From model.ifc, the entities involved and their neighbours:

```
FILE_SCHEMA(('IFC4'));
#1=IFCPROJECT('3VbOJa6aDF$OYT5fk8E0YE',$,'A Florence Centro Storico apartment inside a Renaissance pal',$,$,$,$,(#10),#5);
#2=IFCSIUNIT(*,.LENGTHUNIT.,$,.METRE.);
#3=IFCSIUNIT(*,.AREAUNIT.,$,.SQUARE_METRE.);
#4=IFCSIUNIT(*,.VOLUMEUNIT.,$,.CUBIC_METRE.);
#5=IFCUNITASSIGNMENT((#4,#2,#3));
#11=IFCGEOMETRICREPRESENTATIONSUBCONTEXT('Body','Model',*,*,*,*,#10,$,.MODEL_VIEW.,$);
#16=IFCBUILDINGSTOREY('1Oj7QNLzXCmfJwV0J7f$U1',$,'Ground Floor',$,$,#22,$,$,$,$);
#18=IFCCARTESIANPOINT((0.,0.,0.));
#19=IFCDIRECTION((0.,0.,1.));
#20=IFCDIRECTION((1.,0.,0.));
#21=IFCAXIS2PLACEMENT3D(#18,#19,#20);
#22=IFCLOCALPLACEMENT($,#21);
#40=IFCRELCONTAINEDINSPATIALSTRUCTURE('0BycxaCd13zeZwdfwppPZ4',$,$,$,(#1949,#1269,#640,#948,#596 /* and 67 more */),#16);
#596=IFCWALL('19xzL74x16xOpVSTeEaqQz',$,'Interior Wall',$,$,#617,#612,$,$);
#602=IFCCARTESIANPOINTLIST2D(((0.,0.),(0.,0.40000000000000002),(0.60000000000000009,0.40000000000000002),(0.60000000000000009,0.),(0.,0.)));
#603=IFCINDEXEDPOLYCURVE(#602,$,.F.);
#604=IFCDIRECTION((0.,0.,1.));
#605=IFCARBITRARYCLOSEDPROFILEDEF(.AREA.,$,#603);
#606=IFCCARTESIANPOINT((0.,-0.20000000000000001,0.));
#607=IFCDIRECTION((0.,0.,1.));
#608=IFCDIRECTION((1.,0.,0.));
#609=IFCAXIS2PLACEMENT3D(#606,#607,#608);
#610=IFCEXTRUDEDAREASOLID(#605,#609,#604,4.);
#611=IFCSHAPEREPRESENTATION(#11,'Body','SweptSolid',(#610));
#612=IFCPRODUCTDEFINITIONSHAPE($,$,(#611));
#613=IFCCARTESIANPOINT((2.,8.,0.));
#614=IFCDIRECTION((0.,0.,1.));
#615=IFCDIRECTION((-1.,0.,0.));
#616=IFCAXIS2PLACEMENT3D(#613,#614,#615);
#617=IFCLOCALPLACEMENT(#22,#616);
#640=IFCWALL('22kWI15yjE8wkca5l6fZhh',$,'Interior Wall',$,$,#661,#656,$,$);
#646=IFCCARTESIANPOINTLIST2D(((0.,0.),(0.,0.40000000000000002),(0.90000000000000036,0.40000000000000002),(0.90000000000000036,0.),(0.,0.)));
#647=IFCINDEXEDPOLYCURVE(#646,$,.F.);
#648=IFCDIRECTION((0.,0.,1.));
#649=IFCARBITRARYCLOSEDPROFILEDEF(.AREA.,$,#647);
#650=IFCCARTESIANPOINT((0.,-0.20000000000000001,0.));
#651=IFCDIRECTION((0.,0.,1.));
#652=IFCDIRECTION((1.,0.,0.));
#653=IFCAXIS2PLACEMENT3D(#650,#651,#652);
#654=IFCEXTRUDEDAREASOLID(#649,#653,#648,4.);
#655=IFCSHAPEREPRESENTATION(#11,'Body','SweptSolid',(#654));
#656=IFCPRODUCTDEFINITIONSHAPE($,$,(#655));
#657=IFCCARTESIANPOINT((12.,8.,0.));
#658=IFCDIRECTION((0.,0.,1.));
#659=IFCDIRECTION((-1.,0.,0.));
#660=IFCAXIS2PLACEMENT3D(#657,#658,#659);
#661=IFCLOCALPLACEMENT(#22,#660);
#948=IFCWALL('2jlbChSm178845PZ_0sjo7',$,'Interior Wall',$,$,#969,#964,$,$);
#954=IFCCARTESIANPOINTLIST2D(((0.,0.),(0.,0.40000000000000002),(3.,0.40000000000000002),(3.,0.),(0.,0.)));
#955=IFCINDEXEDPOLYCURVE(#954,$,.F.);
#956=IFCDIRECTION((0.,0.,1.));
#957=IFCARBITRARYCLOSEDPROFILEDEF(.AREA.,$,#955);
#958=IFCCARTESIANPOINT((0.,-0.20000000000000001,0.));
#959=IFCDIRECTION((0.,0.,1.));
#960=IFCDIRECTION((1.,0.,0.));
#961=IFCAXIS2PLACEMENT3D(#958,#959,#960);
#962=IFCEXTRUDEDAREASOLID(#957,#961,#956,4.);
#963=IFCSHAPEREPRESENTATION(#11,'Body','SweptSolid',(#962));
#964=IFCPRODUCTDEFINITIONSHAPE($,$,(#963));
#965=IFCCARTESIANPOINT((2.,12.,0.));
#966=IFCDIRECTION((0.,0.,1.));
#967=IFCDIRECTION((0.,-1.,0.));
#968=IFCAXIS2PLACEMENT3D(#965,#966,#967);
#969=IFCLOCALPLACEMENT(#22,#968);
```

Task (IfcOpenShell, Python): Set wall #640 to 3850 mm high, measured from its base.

```python
import ifcopenshell
import ifcopenshell.geom
import ifcopenshell.util.representation
import ifcopenshell.util.shape

model = ifcopenshell.open("model.ifc")
settings = ifcopenshell.geom.settings()


def volume(element):
    """Net volume in cubic metres, openings subtracted."""
    shape = ifcopenshell.geom.create_shape(settings, element)
    return ifcopenshell.util.shape.get_volume(shape.geometry)


wall = model.by_id(640)
before = volume(wall)

body = ifcopenshell.util.representation.get_representation(wall, "Model", "Body")
solid = body.Items[0]
old_height = solid.Depth
solid.Depth = 3.85
after = volume(wall)

print(f"height {old_height:g} -> {solid.Depth:g}, volume {before:.3f} -> {after:.3f} m3")

model.write("model_edited.ifc")
```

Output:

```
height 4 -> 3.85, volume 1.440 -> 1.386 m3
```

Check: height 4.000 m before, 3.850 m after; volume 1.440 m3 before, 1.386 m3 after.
